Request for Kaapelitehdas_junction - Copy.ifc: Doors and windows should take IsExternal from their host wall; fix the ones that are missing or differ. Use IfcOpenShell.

First a look at what the model holds.

```python
import ifcopenshell
import ifcopenshell.util.element

model = ifcopenshell.open("Kaapelitehdas_junction - Copy.ifc")
print(model.schema)
seen = {}
for e in model.by_type("IfcDoor") + model.by_type("IfcWindow"):
    if not e.FillsVoids:
        continue
    host = e.FillsVoids[0].RelatingOpeningElement.VoidsElements[0].RelatingBuildingElement
    own = ifcopenshell.util.element.get_pset(e, f"Pset_{e.is_a()[3:].removesuffix('StandardCase')}Common", "IsExternal")
    wall = ifcopenshell.util.element.get_pset(host, "Pset_WallCommon", "IsExternal")
    seen[e.is_a(), own, wall] = seen.get((e.is_a(), own, wall), 0) + 1
for (cls, own, wall), count in sorted(seen.items(), key=str):
    print(count, cls, "IsExternal:", own, "| host wall:", wall)
```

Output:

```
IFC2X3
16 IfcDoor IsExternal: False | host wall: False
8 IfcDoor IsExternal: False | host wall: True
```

```python
import ifcopenshell
import ifcopenshell.api.pset
import ifcopenshell.util.element

model = ifcopenshell.open("Kaapelitehdas_junction - Copy.ifc")

count = 0
for ifc_class, pset_name in (("IfcDoor", "Pset_DoorCommon"), ("IfcWindow", "Pset_WindowCommon")):
    for e in model.by_type(ifc_class):
        if not e.FillsVoids:
            continue
        host = e.FillsVoids[0].RelatingOpeningElement.VoidsElements[0].RelatingBuildingElement
        external = ifcopenshell.util.element.get_pset(host, "Pset_WallCommon", "IsExternal")
        if external is None or ifcopenshell.util.element.get_pset(e, pset_name, "IsExternal") == external:
            continue
        pset = ifcopenshell.api.pset.add_pset(model, product=e, name=pset_name)
        ifcopenshell.api.pset.edit_pset(model, pset=pset, properties={"IsExternal": external})
        count += 1

print(count, "updated")

model.write("Kaapelitehdas_junction - Copy_updated.ifc")
```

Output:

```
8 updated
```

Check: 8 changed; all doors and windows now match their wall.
